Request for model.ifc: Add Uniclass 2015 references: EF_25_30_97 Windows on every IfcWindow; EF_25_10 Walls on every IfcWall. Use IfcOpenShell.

First a look at what the model holds.

```python
import ifcopenshell

model = ifcopenshell.open("model.ifc")
print(model.schema)
print("classifications:", [c.Name for c in model.by_type("IfcClassification")])
for ifc_class in ("IfcDoor", "IfcRoof", "IfcStair", "IfcWall", "IfcWindow"):
    print(ifc_class, len(model.by_type(ifc_class)))
```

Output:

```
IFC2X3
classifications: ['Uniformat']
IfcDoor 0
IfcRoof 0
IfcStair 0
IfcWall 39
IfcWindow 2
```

```python
import ifcopenshell
import ifcopenshell.api.classification

model = ifcopenshell.open("model.ifc")

# IFC2X3 requires Source and Edition and has no link from the project to the system.
system = model.create_entity("IfcClassification", Source="NBS", Edition="2015", Name="Uniclass 2015")

codes = {
    "IfcWindow": ("EF_25_30_97", "Windows"),
    "IfcWall": ("EF_25_10", "Walls"),
}
for ifc_class, (code, name) in codes.items():
    products = model.by_type(ifc_class)
    ifcopenshell.api.classification.add_reference(
        model, products=products, classification=system, identification=code, name=name
    )
    print(code, len(products))

model.write("model-out.ifc")
```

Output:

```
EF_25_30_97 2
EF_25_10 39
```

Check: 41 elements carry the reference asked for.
